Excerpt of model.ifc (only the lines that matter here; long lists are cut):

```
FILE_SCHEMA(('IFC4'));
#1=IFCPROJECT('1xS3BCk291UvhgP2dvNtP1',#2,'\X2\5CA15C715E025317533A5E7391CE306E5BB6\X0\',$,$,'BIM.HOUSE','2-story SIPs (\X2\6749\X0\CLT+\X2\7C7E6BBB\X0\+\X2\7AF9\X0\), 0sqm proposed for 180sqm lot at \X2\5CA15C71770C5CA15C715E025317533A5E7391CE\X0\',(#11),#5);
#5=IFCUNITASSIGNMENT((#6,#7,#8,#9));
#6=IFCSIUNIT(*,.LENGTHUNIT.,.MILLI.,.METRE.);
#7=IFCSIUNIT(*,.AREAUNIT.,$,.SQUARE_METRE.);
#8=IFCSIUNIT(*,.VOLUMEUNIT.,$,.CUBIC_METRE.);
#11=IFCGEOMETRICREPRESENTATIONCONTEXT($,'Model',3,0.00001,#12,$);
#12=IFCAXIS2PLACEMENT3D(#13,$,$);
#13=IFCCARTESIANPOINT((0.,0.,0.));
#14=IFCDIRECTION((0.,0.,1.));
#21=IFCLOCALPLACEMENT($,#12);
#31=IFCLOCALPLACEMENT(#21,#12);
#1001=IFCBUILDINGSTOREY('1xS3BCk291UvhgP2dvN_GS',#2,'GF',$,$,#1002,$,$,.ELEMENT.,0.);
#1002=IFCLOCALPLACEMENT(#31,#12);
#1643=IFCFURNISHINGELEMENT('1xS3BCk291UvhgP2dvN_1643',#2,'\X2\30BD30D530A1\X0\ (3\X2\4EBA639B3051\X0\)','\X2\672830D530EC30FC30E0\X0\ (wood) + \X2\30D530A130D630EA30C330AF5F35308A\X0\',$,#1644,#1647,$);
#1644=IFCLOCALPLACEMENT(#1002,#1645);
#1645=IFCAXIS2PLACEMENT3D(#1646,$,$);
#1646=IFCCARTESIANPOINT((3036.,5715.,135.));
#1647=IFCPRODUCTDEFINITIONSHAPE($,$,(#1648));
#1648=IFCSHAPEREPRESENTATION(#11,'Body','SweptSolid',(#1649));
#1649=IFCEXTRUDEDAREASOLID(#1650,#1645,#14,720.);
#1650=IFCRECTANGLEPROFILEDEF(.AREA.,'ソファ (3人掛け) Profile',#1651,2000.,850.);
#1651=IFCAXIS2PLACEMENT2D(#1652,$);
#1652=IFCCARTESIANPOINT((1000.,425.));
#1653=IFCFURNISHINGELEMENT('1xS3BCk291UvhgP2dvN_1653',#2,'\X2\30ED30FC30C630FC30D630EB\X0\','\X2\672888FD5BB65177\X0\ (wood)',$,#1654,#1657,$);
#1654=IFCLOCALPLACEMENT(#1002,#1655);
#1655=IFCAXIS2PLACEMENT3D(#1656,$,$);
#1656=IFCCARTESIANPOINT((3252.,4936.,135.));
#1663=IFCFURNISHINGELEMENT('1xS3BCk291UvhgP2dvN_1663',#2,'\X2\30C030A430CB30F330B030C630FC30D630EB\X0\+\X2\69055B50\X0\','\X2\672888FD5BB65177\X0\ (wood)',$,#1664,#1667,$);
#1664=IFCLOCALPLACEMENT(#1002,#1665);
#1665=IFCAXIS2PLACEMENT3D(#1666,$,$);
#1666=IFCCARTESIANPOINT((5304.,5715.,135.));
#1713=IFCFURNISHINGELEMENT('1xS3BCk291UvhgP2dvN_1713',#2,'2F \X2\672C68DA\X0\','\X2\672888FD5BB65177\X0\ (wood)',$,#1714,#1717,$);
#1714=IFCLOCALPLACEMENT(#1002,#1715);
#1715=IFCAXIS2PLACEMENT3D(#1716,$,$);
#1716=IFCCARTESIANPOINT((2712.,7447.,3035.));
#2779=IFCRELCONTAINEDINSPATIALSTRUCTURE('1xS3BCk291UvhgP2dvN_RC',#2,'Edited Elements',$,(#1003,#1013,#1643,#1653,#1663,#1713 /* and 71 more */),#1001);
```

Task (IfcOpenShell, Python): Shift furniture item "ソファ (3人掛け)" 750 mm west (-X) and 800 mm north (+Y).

```python
import ifcopenshell
import ifcopenshell.api.geometry
import ifcopenshell.util.placement

model = ifcopenshell.open("model.ifc")

item = model.by_id(1643)
matrix = ifcopenshell.util.placement.get_local_placement(item.ObjectPlacement)
matrix[0, 3] -= 750.0
matrix[1, 3] += 800.0
ifcopenshell.api.geometry.edit_object_placement(model, product=item, matrix=matrix, is_si=False)

print(ifcopenshell.util.placement.get_local_placement(item.ObjectPlacement).round(3) + 0.0)

model.write("model_edited.ifc")
```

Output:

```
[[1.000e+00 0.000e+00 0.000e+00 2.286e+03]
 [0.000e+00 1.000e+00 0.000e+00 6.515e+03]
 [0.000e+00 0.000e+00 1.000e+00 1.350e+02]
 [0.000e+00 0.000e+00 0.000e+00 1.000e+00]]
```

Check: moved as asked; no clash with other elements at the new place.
